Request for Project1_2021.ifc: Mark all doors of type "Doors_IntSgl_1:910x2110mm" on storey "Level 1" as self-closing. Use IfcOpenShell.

First a look at what the model holds.

```python
import ifcopenshell
import ifcopenshell.util.element

model = ifcopenshell.open("Project1_2021.ifc")
print(model.schema)
storey = next(s for s in model.by_type("IfcBuildingStorey") if s.Name == "Level 1")
doors = [e for e in ifcopenshell.util.element.get_decomposition(storey) if e.is_a("IfcDoor")]
seen = {}
for e in doors:
    element_type = ifcopenshell.util.element.get_type(e)
    key = (element_type.Name if element_type != e and element_type else None, ifcopenshell.util.element.get_pset(e, "Pset_DoorCommon", "SelfClosing"))
    seen[key] = seen.get(key, 0) + 1
for (name, value), count in sorted(seen.items(), key=str):
    print(count, "x", name, "|", value)
```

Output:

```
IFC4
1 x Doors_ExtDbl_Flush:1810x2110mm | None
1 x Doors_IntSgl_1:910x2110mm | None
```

```python
import ifcopenshell
import ifcopenshell.api.pset
import ifcopenshell.util.element

model = ifcopenshell.open("Project1_2021.ifc")

storey = next(s for s in model.by_type("IfcBuildingStorey") if s.Name == "Level 1")
doors = [e for e in ifcopenshell.util.element.get_decomposition(storey) if e.is_a("IfcDoor")]

count = 0
for e in doors:
    element_type = ifcopenshell.util.element.get_type(e)
    if element_type in (None, e) or element_type.Name != "Doors_IntSgl_1:910x2110mm":
        continue
    # add_pset returns the element's existing set when there is one.
    pset = ifcopenshell.api.pset.add_pset(model, product=e, name="Pset_DoorCommon")
    ifcopenshell.api.pset.edit_pset(model, pset=pset, properties={"SelfClosing": True})
    count += 1

print(count, "doors updated")

model.write("Project1_2021_v2.ifc")
```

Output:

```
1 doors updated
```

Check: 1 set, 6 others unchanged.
